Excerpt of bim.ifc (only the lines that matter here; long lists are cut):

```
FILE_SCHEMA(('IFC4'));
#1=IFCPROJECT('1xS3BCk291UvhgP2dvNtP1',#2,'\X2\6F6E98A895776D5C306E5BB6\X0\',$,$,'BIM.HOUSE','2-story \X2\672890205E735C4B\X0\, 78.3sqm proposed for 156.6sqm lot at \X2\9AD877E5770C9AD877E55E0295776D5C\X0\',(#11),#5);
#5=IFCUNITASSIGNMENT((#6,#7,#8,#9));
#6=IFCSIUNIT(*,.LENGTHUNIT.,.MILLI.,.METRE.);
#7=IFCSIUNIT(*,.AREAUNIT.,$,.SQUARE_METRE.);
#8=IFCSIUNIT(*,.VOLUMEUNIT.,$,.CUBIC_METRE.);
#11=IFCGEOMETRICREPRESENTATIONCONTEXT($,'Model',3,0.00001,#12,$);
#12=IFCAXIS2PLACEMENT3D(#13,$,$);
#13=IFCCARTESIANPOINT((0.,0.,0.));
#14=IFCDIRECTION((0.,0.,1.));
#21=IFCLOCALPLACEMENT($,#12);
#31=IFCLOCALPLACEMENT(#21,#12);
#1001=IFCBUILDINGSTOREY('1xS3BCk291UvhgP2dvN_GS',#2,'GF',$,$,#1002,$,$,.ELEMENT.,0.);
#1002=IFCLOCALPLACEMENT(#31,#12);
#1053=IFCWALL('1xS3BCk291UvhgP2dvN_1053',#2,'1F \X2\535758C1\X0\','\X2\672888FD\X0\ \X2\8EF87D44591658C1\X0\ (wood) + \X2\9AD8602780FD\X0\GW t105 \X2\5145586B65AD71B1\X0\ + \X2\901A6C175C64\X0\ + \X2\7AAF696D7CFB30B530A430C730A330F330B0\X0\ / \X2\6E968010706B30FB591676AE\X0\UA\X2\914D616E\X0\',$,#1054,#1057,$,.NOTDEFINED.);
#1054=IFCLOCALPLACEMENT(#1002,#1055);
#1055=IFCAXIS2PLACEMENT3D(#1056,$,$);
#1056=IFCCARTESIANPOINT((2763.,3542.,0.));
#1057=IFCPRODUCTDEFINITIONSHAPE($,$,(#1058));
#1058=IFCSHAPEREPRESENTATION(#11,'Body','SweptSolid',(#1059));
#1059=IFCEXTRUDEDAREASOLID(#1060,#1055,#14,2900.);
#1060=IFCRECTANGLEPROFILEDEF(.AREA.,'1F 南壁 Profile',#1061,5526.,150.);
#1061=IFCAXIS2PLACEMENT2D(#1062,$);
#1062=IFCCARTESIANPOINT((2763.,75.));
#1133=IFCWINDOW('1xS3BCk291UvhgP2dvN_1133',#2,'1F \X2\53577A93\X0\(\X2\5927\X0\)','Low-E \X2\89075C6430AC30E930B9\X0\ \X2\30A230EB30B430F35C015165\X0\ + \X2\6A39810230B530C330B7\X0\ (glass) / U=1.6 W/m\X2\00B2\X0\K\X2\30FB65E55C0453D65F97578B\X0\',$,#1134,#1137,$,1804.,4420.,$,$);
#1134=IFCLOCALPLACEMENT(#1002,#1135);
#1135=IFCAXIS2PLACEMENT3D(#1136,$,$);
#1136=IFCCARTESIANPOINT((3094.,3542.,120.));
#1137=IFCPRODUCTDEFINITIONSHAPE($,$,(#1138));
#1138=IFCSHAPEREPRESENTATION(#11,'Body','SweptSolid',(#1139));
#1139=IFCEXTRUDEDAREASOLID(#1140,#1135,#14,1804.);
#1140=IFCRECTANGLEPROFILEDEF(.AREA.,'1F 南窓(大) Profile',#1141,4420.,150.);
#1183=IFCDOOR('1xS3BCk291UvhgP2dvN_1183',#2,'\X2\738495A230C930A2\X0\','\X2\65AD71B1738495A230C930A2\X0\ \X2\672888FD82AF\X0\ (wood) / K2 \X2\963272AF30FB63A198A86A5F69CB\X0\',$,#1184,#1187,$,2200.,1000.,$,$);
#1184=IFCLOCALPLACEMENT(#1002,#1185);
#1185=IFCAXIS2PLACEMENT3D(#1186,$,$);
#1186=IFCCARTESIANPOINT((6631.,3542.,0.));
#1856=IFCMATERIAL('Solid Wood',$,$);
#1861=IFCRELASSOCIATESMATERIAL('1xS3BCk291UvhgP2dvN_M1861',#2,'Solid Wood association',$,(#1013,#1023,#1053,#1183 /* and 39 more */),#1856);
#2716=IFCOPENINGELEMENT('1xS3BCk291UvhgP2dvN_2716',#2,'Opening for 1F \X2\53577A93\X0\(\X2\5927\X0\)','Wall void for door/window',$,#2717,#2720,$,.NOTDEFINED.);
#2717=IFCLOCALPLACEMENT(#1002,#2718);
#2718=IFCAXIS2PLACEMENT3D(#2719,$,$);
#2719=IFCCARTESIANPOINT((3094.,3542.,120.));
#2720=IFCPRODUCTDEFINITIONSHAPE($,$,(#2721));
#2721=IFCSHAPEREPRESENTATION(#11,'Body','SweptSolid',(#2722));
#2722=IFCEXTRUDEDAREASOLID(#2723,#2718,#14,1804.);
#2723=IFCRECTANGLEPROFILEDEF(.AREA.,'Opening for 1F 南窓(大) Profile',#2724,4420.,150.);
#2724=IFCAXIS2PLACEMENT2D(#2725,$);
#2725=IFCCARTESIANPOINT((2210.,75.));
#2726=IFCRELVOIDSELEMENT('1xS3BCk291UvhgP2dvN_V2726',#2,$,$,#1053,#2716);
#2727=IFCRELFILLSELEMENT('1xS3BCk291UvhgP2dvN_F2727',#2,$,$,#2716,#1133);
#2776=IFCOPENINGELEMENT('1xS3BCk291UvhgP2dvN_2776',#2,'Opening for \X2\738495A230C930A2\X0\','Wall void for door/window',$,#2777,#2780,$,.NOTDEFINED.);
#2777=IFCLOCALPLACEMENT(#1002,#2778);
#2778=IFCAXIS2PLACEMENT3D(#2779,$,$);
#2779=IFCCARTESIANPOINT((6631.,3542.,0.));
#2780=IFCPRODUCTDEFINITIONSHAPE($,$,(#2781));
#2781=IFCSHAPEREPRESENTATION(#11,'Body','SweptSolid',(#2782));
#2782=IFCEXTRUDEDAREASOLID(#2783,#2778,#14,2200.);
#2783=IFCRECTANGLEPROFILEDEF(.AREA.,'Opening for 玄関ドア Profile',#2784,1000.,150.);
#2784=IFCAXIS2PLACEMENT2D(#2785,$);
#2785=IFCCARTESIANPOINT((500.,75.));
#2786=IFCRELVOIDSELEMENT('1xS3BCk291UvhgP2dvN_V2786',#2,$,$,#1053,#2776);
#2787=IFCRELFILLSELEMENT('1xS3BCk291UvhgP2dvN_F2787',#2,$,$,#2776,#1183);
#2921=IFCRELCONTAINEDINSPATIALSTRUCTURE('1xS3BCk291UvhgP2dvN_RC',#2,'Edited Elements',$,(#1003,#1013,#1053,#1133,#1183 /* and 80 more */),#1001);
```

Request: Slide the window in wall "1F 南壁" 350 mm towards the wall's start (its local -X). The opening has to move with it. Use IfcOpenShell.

```python
import ifcopenshell
import ifcopenshell.api.geometry
import ifcopenshell.util.placement
import ifcopenshell.util.unit

model = ifcopenshell.open("bim.ifc")
unit_scale = ifcopenshell.util.unit.calculate_unit_scale(model)

window = model.by_guid("1xS3BCk291UvhgP2dvN_1133")
opening = window.FillsVoids[0].RelatingOpeningElement
wall = opening.VoidsElements[0].RelatingBuildingElement

wall_matrix = ifcopenshell.util.placement.get_local_placement(wall.ObjectPlacement)
shift = wall_matrix[:3, 0] * -0.35 / unit_scale
before = ifcopenshell.util.placement.get_local_placement(window.ObjectPlacement)[:3, 3].copy()

# The window is not placed relative to its opening, so move both.
for product in (opening, window):
    matrix = ifcopenshell.util.placement.get_local_placement(product.ObjectPlacement)
    matrix[:3, 3] += shift
    ifcopenshell.api.geometry.edit_object_placement(model, product=product, matrix=matrix, is_si=False)

after = ifcopenshell.util.placement.get_local_placement(window.ObjectPlacement)[:3, 3]
print("window moved by", (after - before).round(3) + 0.0)

model.write("bim-out.ifc")
```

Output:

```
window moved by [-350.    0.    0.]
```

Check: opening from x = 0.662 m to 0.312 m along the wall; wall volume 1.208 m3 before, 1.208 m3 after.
